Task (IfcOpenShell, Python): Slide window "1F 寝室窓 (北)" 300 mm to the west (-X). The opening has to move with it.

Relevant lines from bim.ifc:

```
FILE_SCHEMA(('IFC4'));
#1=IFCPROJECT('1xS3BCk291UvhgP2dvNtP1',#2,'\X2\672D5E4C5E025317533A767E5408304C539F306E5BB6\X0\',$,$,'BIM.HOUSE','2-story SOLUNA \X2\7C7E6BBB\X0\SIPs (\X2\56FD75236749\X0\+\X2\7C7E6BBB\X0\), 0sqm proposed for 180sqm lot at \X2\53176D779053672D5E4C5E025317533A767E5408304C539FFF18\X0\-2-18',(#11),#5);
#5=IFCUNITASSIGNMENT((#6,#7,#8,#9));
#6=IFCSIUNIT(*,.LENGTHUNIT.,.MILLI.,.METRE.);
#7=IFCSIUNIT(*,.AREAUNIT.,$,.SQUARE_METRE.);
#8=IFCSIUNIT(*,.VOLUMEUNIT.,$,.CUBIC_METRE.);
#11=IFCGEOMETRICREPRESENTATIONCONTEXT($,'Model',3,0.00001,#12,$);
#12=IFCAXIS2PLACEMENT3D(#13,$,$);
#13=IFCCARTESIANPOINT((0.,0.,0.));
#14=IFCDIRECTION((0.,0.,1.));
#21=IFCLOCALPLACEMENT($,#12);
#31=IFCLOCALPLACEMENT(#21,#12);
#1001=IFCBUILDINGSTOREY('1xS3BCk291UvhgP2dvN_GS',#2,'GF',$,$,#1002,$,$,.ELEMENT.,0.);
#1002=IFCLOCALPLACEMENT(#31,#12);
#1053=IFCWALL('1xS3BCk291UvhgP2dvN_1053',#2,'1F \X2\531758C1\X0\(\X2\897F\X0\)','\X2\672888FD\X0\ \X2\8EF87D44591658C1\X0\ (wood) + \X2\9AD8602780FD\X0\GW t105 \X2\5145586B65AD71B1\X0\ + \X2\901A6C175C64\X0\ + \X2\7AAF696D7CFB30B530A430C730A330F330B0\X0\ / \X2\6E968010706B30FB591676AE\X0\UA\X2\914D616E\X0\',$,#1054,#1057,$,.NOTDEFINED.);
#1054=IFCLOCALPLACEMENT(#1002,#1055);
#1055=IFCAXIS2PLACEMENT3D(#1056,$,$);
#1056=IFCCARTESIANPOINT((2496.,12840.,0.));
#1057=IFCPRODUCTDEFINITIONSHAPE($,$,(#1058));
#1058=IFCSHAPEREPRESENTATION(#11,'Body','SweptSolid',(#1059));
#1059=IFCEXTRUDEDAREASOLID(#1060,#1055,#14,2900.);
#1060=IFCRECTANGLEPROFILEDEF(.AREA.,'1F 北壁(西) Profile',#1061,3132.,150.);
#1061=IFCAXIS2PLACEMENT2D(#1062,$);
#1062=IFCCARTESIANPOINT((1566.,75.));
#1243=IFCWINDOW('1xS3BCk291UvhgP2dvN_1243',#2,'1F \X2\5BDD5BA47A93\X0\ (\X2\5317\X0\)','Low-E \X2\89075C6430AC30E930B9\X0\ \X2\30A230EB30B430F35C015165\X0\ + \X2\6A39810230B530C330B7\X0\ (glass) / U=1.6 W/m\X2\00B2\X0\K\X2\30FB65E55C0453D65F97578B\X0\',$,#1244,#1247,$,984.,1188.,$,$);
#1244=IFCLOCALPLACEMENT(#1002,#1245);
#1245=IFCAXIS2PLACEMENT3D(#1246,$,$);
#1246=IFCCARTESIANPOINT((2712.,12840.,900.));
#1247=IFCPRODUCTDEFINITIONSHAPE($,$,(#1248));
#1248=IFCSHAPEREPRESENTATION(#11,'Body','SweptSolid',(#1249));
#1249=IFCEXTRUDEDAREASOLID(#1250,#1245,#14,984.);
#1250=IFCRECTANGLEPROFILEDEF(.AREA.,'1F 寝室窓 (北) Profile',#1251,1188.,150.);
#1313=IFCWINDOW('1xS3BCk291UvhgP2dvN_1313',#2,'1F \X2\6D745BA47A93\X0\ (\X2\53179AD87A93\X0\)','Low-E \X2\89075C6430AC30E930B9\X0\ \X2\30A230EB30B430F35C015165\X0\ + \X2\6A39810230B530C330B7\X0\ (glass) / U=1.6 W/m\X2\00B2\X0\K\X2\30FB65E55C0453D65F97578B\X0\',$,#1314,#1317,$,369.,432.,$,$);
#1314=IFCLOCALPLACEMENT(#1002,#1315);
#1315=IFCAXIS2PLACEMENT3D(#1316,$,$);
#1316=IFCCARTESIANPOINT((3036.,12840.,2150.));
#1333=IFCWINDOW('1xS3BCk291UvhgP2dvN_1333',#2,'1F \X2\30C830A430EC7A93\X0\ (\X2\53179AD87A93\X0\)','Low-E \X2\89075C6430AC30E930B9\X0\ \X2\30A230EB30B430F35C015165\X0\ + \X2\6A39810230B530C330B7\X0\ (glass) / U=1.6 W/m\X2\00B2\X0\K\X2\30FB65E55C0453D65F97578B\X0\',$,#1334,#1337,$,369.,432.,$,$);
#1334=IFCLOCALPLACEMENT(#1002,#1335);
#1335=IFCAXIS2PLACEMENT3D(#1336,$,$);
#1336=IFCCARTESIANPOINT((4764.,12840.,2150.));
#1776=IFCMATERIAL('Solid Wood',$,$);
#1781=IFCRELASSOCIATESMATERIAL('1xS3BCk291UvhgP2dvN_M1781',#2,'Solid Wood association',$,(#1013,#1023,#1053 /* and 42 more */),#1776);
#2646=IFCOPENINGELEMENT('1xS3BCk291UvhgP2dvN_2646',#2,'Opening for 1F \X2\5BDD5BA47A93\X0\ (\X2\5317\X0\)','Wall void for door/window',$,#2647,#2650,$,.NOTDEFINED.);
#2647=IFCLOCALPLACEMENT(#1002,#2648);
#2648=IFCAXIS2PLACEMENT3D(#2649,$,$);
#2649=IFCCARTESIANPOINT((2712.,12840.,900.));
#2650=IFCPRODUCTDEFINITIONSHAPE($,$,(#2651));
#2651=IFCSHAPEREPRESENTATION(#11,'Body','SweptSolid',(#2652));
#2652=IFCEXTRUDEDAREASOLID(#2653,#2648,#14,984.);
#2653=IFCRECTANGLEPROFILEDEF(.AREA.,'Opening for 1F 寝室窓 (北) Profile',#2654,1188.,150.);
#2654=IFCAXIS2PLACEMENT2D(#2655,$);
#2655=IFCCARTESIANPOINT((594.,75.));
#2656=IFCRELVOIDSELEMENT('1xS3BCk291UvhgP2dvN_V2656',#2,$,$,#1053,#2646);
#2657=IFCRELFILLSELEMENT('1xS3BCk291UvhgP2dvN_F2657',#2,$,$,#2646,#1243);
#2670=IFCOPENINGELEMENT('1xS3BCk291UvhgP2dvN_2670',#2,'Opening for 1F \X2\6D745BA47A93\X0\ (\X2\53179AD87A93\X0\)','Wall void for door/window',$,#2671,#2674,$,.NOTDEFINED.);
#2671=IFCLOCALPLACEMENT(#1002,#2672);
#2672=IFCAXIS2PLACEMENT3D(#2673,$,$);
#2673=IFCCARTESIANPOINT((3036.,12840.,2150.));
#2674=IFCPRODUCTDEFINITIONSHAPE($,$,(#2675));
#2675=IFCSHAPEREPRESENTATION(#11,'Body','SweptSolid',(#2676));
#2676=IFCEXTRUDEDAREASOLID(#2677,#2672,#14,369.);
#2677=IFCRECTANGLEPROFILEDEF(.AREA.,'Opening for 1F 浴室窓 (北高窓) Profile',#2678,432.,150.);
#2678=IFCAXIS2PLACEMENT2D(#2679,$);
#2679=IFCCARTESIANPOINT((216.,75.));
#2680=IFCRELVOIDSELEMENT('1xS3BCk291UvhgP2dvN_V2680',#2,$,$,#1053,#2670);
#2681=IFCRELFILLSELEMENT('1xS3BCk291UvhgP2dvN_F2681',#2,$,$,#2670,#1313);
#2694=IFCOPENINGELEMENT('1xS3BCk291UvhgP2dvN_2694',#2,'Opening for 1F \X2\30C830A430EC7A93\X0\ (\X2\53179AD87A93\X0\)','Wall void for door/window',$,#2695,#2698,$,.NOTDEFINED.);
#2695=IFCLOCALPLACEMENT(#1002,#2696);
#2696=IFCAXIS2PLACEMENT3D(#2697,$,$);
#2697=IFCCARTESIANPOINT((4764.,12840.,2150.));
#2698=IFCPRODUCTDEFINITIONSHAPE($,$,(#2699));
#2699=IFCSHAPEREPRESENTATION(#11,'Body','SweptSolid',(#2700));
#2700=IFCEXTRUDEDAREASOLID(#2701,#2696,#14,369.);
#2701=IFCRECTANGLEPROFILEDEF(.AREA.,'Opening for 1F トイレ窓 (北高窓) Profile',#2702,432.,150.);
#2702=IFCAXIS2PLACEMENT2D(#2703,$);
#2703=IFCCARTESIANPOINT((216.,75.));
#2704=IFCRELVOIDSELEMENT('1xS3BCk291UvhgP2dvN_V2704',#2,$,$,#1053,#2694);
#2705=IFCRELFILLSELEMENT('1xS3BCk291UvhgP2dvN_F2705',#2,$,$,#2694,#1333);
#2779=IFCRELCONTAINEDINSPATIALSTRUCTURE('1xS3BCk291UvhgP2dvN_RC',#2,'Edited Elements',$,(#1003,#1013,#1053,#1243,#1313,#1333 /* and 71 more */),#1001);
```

```python
import ifcopenshell
import ifcopenshell.api.geometry
import ifcopenshell.util.placement

model = ifcopenshell.open("bim.ifc")

window = model.by_guid("1xS3BCk291UvhgP2dvN_1243")
opening = window.FillsVoids[0].RelatingOpeningElement
wall = opening.VoidsElements[0].RelatingBuildingElement

wall_matrix = ifcopenshell.util.placement.get_local_placement(wall.ObjectPlacement)
shift = wall_matrix[:3, 0] * -300.0
before = ifcopenshell.util.placement.get_local_placement(window.ObjectPlacement)[:3, 3].copy()

# The window is not placed relative to its opening, so move both.
for product in (opening, window):
    matrix = ifcopenshell.util.placement.get_local_placement(product.ObjectPlacement)
    matrix[:3, 3] += shift
    ifcopenshell.api.geometry.edit_object_placement(model, product=product, matrix=matrix, is_si=False)

after = ifcopenshell.util.placement.get_local_placement(window.ObjectPlacement)[:3, 3]
print("window moved by", (after - before).round(3) + 0.0)

model.write("bim_v2.ifc")
```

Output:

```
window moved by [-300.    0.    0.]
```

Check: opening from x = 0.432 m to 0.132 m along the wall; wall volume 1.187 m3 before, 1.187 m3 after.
